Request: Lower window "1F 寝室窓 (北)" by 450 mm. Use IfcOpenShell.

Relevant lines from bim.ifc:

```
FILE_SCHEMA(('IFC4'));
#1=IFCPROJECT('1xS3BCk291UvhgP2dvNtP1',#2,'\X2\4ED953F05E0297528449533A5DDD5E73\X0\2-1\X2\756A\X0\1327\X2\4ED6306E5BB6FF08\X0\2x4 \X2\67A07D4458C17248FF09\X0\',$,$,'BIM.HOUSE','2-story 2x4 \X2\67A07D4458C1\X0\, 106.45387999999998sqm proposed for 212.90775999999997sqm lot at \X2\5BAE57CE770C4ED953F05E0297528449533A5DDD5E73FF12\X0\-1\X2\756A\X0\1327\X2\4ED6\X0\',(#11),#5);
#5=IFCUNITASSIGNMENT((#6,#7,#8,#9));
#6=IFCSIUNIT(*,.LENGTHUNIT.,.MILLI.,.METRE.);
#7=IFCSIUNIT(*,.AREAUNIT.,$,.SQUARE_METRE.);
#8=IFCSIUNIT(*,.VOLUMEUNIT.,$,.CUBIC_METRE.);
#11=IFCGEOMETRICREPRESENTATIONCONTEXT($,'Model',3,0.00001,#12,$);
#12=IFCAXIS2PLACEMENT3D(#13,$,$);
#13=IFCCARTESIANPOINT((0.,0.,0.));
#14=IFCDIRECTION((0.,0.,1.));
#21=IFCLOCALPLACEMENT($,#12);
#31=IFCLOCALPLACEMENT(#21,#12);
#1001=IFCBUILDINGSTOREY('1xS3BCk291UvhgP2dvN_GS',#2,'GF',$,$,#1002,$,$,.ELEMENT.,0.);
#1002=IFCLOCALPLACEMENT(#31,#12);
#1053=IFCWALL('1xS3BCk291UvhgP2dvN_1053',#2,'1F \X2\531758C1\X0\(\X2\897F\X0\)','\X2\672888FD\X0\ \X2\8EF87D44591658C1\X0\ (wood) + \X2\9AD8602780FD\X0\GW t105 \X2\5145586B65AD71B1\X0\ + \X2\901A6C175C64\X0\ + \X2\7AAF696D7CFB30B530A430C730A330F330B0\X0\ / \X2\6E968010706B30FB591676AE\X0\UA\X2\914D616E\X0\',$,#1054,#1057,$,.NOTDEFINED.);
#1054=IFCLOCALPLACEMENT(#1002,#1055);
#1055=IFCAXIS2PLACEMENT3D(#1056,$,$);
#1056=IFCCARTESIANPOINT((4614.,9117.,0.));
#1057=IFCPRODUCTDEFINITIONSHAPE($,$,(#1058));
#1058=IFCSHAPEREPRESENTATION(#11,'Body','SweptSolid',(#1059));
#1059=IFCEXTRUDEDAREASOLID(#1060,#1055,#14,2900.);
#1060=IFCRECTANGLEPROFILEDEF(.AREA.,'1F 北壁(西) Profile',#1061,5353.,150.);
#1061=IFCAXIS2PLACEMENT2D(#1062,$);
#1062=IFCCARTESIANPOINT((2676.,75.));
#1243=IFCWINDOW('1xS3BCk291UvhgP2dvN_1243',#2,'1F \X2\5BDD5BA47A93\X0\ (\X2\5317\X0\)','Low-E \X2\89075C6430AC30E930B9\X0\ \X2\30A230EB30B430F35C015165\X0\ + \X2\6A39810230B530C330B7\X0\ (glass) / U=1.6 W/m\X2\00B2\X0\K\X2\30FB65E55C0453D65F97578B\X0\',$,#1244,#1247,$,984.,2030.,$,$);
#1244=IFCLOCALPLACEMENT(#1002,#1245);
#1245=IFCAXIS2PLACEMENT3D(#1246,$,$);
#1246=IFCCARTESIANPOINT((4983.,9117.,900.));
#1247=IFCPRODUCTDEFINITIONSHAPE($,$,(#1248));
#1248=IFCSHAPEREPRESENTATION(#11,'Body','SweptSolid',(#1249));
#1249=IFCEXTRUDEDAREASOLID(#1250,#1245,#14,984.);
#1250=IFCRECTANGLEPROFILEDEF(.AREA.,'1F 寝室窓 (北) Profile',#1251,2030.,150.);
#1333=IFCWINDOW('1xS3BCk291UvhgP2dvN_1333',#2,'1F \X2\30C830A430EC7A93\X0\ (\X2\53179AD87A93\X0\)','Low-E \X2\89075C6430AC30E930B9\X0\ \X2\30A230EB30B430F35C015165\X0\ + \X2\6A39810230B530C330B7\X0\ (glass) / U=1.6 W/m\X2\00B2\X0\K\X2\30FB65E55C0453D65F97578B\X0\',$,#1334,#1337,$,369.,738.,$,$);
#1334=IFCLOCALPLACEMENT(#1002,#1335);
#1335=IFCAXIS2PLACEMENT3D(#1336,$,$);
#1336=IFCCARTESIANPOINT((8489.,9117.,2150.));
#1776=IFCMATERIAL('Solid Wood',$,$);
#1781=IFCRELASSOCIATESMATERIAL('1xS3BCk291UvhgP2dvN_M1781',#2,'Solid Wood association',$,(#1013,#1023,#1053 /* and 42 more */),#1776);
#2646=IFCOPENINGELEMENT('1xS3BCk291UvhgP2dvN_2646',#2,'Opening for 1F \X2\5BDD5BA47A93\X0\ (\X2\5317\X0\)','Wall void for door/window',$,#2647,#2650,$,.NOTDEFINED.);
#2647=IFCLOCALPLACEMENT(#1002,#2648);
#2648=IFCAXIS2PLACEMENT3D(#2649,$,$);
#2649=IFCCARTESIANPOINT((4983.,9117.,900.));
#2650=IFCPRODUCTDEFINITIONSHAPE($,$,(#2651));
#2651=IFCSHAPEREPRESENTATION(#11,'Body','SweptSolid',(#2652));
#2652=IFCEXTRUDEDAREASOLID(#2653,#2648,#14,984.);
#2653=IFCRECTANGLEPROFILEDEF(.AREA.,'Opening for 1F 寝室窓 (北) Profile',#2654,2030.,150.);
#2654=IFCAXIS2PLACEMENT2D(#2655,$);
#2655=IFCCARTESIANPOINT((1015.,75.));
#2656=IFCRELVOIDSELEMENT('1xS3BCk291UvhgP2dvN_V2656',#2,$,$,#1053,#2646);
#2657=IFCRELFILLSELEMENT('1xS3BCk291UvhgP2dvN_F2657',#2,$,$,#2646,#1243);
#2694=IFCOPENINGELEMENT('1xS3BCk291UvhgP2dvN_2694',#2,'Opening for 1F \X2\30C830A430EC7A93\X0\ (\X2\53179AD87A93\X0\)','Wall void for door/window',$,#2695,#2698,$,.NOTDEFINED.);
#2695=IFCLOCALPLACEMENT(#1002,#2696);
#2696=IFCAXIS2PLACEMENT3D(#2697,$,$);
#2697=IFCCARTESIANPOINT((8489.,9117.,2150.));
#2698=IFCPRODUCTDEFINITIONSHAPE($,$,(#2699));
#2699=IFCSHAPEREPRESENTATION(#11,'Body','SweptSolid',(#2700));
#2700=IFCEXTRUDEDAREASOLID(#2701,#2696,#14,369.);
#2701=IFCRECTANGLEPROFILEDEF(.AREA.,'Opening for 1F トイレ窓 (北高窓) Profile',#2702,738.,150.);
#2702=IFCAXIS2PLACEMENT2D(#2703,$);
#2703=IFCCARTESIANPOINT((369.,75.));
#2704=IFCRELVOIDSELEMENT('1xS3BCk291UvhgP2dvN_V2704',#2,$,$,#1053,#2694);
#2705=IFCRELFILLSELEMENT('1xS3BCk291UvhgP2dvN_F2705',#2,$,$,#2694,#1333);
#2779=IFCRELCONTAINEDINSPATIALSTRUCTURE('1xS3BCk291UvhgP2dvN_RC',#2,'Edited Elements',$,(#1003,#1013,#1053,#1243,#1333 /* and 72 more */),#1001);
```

```python
import numpy as np
import ifcopenshell
import ifcopenshell.api.geometry
import ifcopenshell.util.placement
import ifcopenshell.util.unit

model = ifcopenshell.open("bim.ifc")
unit_scale = ifcopenshell.util.unit.calculate_unit_scale(model)

window = model.by_guid("1xS3BCk291UvhgP2dvN_1243")
opening = window.FillsVoids[0].RelatingOpeningElement
dz = -0.45 / unit_scale

shift = np.array([0.0, 0.0, dz])
# The window is not placed relative to its opening, so move both.
for product in (opening, window):
    matrix = ifcopenshell.util.placement.get_local_placement(product.ObjectPlacement)
    matrix[:3, 3] += shift
    ifcopenshell.api.geometry.edit_object_placement(model, product=product, matrix=matrix, is_si=False)

print(f"moved by {dz * unit_scale:+.3f} m")

model.write("bim_edited.ifc")
```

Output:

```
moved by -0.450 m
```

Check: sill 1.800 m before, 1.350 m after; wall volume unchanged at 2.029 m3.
